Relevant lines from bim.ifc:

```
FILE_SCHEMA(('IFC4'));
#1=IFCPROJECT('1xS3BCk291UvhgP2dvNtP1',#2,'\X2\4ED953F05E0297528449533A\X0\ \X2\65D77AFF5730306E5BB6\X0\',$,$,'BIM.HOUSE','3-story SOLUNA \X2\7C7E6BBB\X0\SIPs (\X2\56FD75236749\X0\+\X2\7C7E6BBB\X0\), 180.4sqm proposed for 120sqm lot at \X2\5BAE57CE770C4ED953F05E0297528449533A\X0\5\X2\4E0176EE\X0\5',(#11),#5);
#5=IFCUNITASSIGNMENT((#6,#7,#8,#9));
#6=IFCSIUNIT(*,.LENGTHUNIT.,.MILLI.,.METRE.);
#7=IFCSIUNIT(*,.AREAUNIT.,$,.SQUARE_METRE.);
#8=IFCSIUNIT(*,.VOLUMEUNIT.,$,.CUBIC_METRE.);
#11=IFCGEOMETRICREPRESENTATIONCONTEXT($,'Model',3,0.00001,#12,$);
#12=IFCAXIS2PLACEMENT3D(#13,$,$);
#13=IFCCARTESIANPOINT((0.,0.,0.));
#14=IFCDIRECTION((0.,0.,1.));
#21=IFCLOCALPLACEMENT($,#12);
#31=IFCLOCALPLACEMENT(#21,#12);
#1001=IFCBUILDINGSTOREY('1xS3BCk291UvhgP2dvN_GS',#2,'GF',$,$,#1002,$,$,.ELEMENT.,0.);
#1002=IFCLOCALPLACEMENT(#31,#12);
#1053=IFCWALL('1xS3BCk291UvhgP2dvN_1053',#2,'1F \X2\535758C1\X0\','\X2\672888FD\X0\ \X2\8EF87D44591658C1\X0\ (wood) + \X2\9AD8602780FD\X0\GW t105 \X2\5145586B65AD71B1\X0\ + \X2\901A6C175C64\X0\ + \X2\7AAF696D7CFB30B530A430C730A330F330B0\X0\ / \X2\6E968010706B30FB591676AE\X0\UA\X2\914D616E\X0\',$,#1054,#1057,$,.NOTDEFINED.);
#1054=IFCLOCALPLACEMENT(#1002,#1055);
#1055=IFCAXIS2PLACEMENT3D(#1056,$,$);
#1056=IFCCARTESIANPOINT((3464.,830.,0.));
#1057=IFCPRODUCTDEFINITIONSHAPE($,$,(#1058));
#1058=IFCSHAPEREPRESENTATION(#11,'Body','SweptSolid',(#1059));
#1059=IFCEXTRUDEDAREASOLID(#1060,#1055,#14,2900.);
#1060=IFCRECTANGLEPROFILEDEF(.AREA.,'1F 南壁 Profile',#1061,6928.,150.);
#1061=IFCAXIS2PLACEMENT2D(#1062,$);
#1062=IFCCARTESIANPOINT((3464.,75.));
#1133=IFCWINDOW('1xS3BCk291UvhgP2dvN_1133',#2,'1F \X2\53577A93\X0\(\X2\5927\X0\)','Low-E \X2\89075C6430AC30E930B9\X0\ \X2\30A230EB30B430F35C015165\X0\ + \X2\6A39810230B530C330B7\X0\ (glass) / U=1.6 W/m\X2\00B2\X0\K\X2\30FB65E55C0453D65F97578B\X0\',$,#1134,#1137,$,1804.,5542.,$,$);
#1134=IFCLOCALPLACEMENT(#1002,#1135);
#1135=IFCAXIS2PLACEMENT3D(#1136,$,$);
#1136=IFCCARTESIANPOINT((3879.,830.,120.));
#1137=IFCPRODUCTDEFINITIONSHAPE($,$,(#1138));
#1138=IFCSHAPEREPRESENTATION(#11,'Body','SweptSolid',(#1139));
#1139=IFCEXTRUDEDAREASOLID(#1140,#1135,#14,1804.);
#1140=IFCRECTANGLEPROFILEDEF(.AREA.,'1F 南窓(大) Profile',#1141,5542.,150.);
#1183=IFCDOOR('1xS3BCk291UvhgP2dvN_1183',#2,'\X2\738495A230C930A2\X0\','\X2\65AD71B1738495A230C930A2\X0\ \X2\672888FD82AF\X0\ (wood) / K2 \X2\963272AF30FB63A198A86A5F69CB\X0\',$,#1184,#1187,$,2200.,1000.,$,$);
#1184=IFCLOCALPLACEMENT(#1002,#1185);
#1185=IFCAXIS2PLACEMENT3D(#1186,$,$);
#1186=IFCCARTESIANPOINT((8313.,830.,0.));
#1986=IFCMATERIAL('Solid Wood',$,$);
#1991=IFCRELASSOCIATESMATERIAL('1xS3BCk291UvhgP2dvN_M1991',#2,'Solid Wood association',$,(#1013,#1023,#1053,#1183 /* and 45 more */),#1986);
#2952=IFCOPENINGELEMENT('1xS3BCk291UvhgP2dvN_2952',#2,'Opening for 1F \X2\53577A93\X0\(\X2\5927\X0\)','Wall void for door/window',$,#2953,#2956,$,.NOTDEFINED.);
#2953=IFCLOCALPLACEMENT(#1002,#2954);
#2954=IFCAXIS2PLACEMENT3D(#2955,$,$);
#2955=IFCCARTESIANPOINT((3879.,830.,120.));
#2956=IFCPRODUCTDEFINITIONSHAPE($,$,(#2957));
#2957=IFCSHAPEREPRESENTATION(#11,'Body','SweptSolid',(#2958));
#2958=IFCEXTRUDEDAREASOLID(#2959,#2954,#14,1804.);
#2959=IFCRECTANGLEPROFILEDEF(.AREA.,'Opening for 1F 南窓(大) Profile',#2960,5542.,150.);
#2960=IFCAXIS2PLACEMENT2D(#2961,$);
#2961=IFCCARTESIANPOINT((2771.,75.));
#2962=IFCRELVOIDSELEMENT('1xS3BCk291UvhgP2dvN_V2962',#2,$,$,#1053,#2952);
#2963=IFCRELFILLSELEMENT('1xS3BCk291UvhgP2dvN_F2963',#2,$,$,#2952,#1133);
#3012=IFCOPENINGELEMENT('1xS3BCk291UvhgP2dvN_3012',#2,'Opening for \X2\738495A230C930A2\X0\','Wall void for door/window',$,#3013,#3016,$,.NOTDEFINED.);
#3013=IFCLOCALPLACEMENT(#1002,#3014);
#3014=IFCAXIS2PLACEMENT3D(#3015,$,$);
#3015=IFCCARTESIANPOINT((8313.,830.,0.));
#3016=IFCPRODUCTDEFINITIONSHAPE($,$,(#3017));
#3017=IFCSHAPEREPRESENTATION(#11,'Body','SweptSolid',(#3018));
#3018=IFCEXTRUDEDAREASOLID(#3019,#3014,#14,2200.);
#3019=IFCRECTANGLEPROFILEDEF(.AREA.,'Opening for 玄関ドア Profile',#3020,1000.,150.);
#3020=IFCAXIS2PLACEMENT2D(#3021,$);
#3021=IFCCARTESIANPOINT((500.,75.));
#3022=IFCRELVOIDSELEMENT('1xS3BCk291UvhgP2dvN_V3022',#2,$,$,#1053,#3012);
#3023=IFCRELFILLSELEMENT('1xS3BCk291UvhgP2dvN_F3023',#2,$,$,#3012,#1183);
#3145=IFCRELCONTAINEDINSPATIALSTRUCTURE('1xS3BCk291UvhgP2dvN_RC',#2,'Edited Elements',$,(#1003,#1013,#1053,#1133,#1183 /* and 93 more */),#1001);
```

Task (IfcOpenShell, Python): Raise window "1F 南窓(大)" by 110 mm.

```python
import numpy as np
import ifcopenshell
import ifcopenshell.api.geometry
import ifcopenshell.util.placement
import ifcopenshell.util.unit

model = ifcopenshell.open("bim.ifc")
unit_scale = ifcopenshell.util.unit.calculate_unit_scale(model)

window = model.by_guid("1xS3BCk291UvhgP2dvN_1133")
opening = window.FillsVoids[0].RelatingOpeningElement
dz = 110.0

shift = np.array([0.0, 0.0, dz])
# The window is not placed relative to its opening, so move both.
for product in (opening, window):
    matrix = ifcopenshell.util.placement.get_local_placement(product.ObjectPlacement)
    matrix[:3, 3] += shift
    ifcopenshell.api.geometry.edit_object_placement(model, product=product, matrix=matrix, is_si=False)

print(f"moved by {dz * unit_scale:+.3f} m")

model.write("bim_rev.ifc")
```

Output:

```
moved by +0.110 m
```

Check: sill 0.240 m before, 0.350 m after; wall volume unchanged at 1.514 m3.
